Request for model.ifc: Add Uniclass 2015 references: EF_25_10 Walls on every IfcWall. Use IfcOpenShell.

First a look at what the model holds.

```python
import ifcopenshell

model = ifcopenshell.open("model.ifc")
print(model.schema)
print("classifications:", [c.Name for c in model.by_type("IfcClassification")])
for ifc_class in ("IfcDoor", "IfcRoof", "IfcStair", "IfcWall", "IfcWindow"):
    print(ifc_class, len(model.by_type(ifc_class)))
```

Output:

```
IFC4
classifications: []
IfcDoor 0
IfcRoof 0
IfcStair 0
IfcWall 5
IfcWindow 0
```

```python
import ifcopenshell
import ifcopenshell.api.classification

model = ifcopenshell.open("model.ifc")

system = ifcopenshell.api.classification.add_classification(model, classification="Uniclass 2015")

codes = {
    "IfcWall": ("EF_25_10", "Walls"),
}
for ifc_class, (code, name) in codes.items():
    products = model.by_type(ifc_class)
    ifcopenshell.api.classification.add_reference(
        model, products=products, classification=system, identification=code, name=name
    )
    print(code, len(products))

model.write("model_updated.ifc")
```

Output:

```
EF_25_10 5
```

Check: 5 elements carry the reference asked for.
